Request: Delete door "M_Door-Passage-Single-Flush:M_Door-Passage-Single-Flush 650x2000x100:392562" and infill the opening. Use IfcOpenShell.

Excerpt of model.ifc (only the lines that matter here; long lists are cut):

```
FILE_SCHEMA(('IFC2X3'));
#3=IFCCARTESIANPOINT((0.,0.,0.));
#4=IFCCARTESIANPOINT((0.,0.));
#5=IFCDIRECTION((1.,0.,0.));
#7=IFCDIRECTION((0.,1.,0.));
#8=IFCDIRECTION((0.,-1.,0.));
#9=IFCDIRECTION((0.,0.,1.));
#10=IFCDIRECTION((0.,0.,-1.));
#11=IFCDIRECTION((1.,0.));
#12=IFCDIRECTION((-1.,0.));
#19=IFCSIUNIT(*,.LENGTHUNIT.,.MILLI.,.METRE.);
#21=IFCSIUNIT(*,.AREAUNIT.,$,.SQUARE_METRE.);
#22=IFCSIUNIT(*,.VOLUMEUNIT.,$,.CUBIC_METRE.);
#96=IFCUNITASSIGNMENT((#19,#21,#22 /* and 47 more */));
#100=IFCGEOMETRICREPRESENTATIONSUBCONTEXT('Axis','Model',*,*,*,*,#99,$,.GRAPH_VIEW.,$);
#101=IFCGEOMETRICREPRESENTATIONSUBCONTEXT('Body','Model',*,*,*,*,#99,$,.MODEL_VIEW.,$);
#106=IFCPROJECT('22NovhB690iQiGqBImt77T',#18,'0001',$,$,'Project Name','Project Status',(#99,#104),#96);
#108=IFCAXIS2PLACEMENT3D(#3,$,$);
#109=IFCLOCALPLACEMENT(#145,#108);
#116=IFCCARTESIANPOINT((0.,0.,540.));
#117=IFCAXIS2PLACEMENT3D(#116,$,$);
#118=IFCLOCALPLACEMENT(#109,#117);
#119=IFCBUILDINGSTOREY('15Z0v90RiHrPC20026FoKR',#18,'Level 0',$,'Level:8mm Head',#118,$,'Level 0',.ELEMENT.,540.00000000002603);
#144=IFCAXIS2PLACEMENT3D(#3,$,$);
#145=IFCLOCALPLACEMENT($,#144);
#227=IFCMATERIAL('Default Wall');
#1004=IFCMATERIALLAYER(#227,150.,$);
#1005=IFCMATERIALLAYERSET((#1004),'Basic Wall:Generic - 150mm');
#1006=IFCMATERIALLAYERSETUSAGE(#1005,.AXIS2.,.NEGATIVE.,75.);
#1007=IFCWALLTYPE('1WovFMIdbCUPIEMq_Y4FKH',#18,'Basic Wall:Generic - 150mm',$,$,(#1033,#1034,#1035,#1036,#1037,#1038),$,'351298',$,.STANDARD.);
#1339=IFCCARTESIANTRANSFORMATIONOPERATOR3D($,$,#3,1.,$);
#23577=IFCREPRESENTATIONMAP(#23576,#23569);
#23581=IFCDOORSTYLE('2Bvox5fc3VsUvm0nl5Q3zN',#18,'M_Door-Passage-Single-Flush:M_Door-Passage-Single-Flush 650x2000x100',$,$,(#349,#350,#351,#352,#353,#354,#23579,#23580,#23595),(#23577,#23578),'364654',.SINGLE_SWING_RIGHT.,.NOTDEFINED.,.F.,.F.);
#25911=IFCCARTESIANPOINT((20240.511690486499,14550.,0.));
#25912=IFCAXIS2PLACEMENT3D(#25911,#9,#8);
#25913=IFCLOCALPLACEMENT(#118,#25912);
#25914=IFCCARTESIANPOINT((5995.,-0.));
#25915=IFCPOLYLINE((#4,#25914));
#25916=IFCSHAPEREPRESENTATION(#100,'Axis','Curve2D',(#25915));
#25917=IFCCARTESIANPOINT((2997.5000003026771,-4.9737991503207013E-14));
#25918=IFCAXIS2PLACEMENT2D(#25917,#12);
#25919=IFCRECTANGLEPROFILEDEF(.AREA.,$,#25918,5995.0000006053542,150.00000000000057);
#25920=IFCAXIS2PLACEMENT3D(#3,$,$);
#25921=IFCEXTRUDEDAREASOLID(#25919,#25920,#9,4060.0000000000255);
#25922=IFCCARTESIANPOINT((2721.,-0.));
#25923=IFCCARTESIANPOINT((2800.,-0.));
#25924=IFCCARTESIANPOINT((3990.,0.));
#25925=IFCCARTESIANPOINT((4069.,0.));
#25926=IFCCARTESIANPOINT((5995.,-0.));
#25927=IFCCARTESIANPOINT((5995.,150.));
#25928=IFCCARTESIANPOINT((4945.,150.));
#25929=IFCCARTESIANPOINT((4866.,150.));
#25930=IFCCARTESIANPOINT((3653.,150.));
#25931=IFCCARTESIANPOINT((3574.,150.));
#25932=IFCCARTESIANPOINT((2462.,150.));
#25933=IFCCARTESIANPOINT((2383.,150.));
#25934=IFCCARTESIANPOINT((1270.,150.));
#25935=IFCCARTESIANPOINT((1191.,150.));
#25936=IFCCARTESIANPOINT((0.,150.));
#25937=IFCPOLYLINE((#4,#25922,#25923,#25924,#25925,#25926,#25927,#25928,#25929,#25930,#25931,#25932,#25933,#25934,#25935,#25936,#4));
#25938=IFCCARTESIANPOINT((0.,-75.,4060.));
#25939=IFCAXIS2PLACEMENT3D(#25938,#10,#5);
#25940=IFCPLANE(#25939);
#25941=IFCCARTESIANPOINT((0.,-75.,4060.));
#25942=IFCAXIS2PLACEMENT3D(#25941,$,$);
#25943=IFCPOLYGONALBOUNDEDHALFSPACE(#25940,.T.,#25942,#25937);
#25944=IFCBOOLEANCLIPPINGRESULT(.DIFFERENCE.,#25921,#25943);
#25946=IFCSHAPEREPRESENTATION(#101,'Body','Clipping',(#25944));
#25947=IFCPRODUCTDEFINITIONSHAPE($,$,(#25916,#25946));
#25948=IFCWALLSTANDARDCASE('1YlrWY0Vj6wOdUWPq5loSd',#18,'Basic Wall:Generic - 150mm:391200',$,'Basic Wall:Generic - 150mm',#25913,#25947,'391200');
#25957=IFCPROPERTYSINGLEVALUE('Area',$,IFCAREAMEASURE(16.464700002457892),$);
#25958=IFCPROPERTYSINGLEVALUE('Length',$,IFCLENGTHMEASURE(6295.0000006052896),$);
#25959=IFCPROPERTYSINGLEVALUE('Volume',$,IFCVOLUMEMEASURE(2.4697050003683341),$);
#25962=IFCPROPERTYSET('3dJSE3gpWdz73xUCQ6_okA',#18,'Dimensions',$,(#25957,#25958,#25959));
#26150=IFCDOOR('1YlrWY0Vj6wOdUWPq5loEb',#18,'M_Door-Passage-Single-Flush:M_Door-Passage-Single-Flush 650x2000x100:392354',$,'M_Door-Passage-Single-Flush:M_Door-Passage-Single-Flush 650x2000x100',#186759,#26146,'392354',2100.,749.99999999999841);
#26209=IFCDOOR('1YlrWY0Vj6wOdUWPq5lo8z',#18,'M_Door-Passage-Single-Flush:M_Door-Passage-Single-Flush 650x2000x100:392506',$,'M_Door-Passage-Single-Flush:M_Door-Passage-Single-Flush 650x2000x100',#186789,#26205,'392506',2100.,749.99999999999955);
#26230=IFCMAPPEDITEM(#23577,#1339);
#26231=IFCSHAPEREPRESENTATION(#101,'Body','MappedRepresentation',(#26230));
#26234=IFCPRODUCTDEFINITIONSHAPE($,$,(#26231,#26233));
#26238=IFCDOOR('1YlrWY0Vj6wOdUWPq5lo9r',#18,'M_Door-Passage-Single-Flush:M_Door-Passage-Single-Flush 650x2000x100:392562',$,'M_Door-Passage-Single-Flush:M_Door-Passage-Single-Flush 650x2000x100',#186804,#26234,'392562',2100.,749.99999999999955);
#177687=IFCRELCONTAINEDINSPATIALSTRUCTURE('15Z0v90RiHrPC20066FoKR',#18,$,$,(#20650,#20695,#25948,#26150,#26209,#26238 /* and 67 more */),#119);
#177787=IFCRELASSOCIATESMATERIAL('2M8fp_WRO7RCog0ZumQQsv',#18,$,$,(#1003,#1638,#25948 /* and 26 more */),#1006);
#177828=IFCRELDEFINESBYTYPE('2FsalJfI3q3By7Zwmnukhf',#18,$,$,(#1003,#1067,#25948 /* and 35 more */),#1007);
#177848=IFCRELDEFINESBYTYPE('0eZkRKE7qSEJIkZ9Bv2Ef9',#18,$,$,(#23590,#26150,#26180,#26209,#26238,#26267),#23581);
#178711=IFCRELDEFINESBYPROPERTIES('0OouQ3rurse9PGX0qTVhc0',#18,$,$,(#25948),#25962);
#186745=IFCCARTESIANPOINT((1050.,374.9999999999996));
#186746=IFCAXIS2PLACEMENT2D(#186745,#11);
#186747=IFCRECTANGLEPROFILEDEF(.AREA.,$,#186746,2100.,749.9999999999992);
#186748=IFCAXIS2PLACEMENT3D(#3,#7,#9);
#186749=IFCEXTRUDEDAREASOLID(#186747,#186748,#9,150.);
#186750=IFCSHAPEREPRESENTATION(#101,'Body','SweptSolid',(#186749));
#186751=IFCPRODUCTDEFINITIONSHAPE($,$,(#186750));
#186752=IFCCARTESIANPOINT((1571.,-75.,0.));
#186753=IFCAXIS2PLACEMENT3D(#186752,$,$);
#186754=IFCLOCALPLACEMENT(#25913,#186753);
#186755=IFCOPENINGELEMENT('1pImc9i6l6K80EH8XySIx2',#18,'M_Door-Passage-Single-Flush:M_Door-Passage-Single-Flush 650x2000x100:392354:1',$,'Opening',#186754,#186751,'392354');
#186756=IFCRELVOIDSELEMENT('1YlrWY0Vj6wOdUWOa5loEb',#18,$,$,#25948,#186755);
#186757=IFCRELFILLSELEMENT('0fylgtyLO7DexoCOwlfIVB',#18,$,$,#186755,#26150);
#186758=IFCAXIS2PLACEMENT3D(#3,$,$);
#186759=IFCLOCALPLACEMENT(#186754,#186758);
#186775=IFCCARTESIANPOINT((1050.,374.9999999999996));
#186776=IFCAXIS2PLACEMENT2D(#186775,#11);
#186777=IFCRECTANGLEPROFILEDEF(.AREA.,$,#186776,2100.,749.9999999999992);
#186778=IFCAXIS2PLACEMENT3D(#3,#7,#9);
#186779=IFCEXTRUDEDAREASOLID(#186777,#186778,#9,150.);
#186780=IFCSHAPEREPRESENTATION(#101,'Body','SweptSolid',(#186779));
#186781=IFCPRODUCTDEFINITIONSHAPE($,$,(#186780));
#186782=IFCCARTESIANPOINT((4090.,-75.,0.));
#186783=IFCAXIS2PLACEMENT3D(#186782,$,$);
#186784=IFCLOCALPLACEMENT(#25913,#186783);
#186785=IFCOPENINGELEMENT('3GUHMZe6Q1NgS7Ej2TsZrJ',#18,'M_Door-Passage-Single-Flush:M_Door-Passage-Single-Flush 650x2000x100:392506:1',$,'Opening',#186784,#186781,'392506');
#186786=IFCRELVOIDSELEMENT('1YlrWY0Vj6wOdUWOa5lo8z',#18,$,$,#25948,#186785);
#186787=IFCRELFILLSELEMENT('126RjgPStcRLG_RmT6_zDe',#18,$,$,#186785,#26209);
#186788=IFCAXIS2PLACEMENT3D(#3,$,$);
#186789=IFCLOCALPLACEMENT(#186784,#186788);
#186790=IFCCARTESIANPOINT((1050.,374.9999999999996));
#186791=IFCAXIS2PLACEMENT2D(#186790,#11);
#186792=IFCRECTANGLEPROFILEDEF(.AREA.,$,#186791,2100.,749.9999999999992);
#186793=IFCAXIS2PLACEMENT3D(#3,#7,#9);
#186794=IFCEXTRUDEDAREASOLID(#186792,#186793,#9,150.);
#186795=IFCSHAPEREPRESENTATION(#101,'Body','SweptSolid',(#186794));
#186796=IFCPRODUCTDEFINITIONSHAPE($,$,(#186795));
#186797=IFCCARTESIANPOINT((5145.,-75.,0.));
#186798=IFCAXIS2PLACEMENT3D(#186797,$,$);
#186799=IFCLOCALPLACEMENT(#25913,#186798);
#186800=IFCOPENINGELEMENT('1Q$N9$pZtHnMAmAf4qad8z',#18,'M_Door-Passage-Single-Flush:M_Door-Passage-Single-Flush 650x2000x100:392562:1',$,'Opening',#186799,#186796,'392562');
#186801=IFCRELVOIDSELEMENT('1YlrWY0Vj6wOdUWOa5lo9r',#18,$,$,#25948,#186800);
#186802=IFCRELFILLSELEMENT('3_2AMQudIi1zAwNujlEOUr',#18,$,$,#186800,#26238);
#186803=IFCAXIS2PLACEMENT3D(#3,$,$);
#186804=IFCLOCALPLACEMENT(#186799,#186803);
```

```python
import ifcopenshell
import ifcopenshell.api.feature
import ifcopenshell.api.pset
import ifcopenshell.api.root
import ifcopenshell.geom
import ifcopenshell.util.element
import ifcopenshell.util.shape
import ifcopenshell.util.unit

model = ifcopenshell.open("model.ifc")
area_scale = ifcopenshell.util.unit.calculate_unit_scale(model, "AREAUNIT")
volume_scale = ifcopenshell.util.unit.calculate_unit_scale(model, "VOLUMEUNIT")
settings = ifcopenshell.geom.settings()


def volume(element):
    """Net volume in cubic metres, openings subtracted."""
    shape = ifcopenshell.geom.create_shape(settings, element)
    return ifcopenshell.util.shape.get_volume(shape.geometry)


door = model.by_guid("1YlrWY0Vj6wOdUWPq5lo9r")
opening = door.FillsVoids[0].RelatingOpeningElement
wall = opening.VoidsElements[0].RelatingBuildingElement
before = volume(wall)

ifcopenshell.api.root.remove_product(model, product=door)
ifcopenshell.api.feature.remove_feature(model, feature=opening)

after = volume(wall)
thickness = 0.15  # wall thickness in metres

# Update the wall's stored quantities.
pset = model.by_id(ifcopenshell.util.element.get_pset(wall, "Dimensions", should_inherit=False)["id"])
ifcopenshell.api.pset.edit_pset(model, pset=pset, properties={
    "Area": model.create_entity("IfcAreaMeasure", after / thickness / area_scale),
    "Volume": model.create_entity("IfcVolumeMeasure", after / volume_scale),
})

print(f"wall volume {before:.3f} -> {after:.3f} m3")

model.write("model_edited.ifc")
```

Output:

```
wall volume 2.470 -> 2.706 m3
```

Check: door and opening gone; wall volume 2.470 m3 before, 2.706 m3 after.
